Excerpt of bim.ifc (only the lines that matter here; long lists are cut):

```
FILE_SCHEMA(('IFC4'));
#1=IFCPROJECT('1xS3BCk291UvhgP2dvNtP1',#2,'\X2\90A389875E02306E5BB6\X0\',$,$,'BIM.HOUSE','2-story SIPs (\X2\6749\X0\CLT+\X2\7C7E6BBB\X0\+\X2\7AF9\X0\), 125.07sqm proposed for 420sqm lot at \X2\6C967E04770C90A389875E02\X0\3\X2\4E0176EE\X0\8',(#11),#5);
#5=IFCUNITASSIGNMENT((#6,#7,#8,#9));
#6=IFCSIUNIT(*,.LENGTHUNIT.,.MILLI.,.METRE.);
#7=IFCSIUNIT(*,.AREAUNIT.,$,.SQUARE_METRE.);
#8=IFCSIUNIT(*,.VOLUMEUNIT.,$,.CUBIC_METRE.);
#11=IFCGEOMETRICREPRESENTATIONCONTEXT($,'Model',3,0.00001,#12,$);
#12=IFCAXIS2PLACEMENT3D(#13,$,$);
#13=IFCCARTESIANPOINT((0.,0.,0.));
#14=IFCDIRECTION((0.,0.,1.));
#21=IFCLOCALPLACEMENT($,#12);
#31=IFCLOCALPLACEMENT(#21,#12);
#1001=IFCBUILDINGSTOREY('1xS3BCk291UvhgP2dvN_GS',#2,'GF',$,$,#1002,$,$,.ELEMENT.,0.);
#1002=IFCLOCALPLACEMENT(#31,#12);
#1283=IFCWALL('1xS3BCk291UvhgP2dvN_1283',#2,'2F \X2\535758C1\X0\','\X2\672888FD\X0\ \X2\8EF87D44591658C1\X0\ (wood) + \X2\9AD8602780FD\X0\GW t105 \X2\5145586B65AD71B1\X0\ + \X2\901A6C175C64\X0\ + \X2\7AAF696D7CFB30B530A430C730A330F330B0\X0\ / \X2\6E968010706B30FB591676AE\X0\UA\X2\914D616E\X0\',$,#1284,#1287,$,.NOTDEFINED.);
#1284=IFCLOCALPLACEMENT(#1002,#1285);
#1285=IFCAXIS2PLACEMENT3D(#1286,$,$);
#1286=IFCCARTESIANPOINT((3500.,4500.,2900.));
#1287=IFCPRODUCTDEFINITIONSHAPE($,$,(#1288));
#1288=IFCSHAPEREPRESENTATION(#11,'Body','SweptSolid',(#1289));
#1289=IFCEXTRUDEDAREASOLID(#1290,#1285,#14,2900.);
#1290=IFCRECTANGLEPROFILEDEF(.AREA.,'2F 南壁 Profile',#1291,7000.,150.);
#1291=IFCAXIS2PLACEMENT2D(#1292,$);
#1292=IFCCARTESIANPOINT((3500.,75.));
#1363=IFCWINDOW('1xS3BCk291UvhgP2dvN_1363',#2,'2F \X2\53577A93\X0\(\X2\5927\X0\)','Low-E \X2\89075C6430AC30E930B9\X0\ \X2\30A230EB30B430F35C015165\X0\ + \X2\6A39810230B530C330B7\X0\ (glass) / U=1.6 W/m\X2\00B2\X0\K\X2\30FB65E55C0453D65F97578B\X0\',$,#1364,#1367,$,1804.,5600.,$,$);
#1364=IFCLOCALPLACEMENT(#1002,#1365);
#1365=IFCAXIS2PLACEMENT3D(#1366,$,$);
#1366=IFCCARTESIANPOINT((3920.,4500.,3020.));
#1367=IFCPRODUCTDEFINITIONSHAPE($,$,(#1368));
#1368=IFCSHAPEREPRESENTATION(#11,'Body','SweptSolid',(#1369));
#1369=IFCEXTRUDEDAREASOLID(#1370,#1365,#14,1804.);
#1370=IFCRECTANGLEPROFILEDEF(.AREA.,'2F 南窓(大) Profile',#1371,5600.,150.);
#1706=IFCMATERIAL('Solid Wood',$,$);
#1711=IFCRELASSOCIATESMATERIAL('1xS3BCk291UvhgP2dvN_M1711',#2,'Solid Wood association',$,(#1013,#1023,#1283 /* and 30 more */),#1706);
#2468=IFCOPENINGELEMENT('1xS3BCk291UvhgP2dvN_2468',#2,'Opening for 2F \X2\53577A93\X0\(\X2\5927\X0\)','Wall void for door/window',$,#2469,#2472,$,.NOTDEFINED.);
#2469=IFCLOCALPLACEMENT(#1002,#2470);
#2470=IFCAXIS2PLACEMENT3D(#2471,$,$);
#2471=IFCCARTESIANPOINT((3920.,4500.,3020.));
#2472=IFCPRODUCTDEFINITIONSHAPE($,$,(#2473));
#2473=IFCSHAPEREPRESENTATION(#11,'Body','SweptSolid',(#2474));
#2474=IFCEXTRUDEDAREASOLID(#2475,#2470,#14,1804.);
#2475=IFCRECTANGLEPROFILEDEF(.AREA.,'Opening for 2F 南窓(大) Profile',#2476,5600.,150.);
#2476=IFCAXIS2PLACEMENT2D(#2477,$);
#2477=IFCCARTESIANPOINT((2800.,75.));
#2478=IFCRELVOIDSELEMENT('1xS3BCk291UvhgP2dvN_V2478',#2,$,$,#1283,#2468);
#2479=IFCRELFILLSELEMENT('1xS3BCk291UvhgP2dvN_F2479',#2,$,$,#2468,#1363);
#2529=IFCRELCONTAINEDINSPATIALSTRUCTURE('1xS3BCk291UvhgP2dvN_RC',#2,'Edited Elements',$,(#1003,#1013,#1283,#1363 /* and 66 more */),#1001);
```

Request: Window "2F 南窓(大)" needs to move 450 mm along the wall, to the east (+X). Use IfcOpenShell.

```python
import ifcopenshell
import ifcopenshell.api.geometry
import ifcopenshell.util.placement
import ifcopenshell.util.unit

model = ifcopenshell.open("bim.ifc")
unit_scale = ifcopenshell.util.unit.calculate_unit_scale(model)

window = model.by_id(1363)
opening = window.FillsVoids[0].RelatingOpeningElement
wall = opening.VoidsElements[0].RelatingBuildingElement

wall_matrix = ifcopenshell.util.placement.get_local_placement(wall.ObjectPlacement)
shift = wall_matrix[:3, 0] * 0.45 / unit_scale
before = ifcopenshell.util.placement.get_local_placement(window.ObjectPlacement)[:3, 3].copy()

# The window is not placed relative to its opening, so move both.
for product in (opening, window):
    matrix = ifcopenshell.util.placement.get_local_placement(product.ObjectPlacement)
    matrix[:3, 3] += shift
    ifcopenshell.api.geometry.edit_object_placement(model, product=product, matrix=matrix, is_si=False)

after = ifcopenshell.util.placement.get_local_placement(window.ObjectPlacement)[:3, 3]
print("window moved by", (after - before).round(3) + 0.0)

model.write("bim_edited.ifc")
```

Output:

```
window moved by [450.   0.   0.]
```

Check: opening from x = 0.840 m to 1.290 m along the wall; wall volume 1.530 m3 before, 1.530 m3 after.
